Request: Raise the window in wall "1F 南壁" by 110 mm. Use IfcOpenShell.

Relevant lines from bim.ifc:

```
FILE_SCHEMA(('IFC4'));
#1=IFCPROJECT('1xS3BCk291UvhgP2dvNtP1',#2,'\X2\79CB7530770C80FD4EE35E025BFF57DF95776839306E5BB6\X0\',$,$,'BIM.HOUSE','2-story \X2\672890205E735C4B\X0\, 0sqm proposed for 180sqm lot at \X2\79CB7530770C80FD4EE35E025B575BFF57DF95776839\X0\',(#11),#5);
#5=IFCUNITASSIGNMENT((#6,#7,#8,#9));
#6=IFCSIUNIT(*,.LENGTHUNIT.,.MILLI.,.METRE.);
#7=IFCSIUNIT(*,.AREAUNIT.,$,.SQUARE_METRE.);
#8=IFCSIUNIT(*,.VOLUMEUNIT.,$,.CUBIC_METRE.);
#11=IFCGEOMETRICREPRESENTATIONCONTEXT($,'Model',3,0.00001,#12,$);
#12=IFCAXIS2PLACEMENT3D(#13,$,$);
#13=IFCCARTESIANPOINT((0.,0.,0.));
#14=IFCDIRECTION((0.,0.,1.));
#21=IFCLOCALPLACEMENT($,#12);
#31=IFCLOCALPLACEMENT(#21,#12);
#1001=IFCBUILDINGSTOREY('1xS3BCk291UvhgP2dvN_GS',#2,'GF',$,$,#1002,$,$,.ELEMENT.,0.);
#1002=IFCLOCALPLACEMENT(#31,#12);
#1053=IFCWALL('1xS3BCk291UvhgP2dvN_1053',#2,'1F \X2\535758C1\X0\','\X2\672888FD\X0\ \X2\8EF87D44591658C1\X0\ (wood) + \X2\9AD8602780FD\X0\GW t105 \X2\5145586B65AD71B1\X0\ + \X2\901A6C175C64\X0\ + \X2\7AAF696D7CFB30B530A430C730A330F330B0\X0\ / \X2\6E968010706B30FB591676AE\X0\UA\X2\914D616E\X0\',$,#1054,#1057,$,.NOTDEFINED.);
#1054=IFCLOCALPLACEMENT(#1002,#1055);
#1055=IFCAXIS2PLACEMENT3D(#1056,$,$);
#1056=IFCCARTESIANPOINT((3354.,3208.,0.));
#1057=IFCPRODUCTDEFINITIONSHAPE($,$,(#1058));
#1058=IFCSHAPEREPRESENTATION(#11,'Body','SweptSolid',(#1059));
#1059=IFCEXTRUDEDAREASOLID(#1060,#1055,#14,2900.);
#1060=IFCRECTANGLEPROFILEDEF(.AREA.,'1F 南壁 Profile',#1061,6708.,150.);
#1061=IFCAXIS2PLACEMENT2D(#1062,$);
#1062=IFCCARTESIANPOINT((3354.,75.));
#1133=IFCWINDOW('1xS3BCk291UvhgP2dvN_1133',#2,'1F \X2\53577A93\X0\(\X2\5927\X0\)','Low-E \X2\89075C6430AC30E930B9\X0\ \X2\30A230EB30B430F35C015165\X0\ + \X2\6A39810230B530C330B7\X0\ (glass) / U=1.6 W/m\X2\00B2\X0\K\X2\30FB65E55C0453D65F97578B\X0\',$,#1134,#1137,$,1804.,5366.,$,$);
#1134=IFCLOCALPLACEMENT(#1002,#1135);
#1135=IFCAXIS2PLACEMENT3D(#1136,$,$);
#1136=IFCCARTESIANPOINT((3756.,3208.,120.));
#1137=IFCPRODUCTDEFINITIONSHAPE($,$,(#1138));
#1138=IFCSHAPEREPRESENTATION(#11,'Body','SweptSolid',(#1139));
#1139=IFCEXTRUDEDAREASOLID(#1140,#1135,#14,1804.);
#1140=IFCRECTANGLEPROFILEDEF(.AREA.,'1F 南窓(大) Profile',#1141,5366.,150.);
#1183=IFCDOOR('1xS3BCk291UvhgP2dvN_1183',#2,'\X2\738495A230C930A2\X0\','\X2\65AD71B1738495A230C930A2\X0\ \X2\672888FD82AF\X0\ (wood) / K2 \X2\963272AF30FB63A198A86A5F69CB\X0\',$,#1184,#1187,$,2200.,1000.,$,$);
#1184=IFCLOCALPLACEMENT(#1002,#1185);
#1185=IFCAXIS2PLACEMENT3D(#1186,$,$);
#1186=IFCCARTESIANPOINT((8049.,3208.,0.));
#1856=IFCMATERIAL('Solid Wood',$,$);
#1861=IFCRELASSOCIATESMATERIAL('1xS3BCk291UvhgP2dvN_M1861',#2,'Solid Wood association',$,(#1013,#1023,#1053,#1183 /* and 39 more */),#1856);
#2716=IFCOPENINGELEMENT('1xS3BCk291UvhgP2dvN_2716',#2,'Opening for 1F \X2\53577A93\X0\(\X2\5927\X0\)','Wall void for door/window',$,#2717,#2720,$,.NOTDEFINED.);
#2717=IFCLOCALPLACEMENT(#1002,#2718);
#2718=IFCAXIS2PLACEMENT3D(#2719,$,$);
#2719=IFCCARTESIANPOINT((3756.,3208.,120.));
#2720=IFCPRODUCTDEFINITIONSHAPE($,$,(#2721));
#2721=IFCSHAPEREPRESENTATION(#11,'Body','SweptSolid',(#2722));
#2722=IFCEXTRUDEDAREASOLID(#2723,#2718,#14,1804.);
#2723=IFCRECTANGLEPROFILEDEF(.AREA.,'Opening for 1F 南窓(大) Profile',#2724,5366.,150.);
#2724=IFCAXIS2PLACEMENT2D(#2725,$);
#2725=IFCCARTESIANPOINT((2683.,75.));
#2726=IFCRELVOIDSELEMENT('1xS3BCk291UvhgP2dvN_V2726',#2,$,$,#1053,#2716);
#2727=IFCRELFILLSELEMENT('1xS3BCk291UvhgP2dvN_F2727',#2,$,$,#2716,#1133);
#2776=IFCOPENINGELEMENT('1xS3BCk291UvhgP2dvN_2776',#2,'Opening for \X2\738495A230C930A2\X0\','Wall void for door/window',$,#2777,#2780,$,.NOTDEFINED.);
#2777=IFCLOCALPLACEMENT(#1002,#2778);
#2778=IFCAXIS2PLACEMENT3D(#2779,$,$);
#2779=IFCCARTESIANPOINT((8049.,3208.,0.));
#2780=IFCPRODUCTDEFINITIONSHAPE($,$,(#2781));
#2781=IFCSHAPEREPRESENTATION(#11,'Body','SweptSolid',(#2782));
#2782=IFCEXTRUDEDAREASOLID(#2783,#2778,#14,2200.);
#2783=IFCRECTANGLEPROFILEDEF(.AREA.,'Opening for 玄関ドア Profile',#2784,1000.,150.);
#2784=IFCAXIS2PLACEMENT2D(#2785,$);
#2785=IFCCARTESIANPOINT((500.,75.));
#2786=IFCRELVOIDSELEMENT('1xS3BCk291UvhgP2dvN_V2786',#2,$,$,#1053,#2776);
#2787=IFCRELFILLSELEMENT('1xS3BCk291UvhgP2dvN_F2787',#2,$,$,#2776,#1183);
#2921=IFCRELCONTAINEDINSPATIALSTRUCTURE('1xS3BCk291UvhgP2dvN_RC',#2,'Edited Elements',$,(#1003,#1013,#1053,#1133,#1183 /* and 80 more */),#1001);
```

```python
import numpy as np
import ifcopenshell
import ifcopenshell.api.geometry
import ifcopenshell.util.placement
import ifcopenshell.util.unit

model = ifcopenshell.open("bim.ifc")
unit_scale = ifcopenshell.util.unit.calculate_unit_scale(model)

window = model.by_guid("1xS3BCk291UvhgP2dvN_1133")
opening = window.FillsVoids[0].RelatingOpeningElement
dz = 110.0

shift = np.array([0.0, 0.0, dz])
# The window is not placed relative to its opening, so move both.
for product in (opening, window):
    matrix = ifcopenshell.util.placement.get_local_placement(product.ObjectPlacement)
    matrix[:3, 3] += shift
    ifcopenshell.api.geometry.edit_object_placement(model, product=product, matrix=matrix, is_si=False)

print(f"moved by {dz * unit_scale:+.3f} m")

model.write("bim_updated.ifc")
```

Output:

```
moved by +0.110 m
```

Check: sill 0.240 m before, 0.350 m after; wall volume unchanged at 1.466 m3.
